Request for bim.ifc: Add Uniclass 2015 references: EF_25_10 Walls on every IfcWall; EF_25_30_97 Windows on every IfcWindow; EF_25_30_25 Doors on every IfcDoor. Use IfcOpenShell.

First a look at what the model holds.

```python
import ifcopenshell

model = ifcopenshell.open("bim.ifc")
print(model.schema)
print("classifications:", [c.Name for c in model.by_type("IfcClassification")])
for ifc_class in ("IfcDoor", "IfcRoof", "IfcStair", "IfcWall", "IfcWindow"):
    print(ifc_class, len(model.by_type(ifc_class)))
```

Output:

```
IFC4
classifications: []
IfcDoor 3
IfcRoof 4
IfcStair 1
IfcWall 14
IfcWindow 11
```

```python
import ifcopenshell
import ifcopenshell.api.classification

model = ifcopenshell.open("bim.ifc")

system = ifcopenshell.api.classification.add_classification(model, classification="Uniclass 2015")

codes = {
    "IfcWall": ("EF_25_10", "Walls"),
    "IfcWindow": ("EF_25_30_97", "Windows"),
    "IfcDoor": ("EF_25_30_25", "Doors"),
}
for ifc_class, (code, name) in codes.items():
    products = model.by_type(ifc_class)
    ifcopenshell.api.classification.add_reference(
        model, products=products, classification=system, identification=code, name=name
    )
    print(code, len(products))

model.write("bim_rev.ifc")
```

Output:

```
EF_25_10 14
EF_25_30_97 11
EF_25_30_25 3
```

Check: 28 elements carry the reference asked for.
